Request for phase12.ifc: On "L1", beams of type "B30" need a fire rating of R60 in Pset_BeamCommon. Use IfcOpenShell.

First a look at what the model holds.

```python
import ifcopenshell
import ifcopenshell.util.element

model = ifcopenshell.open("phase12.ifc")
print(model.schema)
storey = next(s for s in model.by_type("IfcBuildingStorey") if s.Name == "L1")
beams = [e for e in ifcopenshell.util.element.get_decomposition(storey) if e.is_a("IfcBeam")]
seen = {}
for e in beams:
    element_type = ifcopenshell.util.element.get_type(e)
    key = (element_type.Name if element_type != e and element_type else None, ifcopenshell.util.element.get_pset(e, "Pset_BeamCommon", "FireRating"))
    seen[key] = seen.get(key, 0) + 1
for (name, value), count in sorted(seen.items(), key=str):
    print(count, "x", name, "|", value)
```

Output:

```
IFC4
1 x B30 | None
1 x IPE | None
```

```python
import ifcopenshell
import ifcopenshell.api.pset
import ifcopenshell.util.element

model = ifcopenshell.open("phase12.ifc")

storey = next(s for s in model.by_type("IfcBuildingStorey") if s.Name == "L1")
beams = [e for e in ifcopenshell.util.element.get_decomposition(storey) if e.is_a("IfcBeam")]

count = 0
for e in beams:
    element_type = ifcopenshell.util.element.get_type(e)
    if element_type in (None, e) or element_type.Name != "B30":
        continue
    # add_pset returns the element's existing set when there is one.
    pset = ifcopenshell.api.pset.add_pset(model, product=e, name="Pset_BeamCommon")
    ifcopenshell.api.pset.edit_pset(model, pset=pset, properties={"FireRating": "R60"})
    count += 1

print(count, "beams updated")

model.write("phase12_rev.ifc")
```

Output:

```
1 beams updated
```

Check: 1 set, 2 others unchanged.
